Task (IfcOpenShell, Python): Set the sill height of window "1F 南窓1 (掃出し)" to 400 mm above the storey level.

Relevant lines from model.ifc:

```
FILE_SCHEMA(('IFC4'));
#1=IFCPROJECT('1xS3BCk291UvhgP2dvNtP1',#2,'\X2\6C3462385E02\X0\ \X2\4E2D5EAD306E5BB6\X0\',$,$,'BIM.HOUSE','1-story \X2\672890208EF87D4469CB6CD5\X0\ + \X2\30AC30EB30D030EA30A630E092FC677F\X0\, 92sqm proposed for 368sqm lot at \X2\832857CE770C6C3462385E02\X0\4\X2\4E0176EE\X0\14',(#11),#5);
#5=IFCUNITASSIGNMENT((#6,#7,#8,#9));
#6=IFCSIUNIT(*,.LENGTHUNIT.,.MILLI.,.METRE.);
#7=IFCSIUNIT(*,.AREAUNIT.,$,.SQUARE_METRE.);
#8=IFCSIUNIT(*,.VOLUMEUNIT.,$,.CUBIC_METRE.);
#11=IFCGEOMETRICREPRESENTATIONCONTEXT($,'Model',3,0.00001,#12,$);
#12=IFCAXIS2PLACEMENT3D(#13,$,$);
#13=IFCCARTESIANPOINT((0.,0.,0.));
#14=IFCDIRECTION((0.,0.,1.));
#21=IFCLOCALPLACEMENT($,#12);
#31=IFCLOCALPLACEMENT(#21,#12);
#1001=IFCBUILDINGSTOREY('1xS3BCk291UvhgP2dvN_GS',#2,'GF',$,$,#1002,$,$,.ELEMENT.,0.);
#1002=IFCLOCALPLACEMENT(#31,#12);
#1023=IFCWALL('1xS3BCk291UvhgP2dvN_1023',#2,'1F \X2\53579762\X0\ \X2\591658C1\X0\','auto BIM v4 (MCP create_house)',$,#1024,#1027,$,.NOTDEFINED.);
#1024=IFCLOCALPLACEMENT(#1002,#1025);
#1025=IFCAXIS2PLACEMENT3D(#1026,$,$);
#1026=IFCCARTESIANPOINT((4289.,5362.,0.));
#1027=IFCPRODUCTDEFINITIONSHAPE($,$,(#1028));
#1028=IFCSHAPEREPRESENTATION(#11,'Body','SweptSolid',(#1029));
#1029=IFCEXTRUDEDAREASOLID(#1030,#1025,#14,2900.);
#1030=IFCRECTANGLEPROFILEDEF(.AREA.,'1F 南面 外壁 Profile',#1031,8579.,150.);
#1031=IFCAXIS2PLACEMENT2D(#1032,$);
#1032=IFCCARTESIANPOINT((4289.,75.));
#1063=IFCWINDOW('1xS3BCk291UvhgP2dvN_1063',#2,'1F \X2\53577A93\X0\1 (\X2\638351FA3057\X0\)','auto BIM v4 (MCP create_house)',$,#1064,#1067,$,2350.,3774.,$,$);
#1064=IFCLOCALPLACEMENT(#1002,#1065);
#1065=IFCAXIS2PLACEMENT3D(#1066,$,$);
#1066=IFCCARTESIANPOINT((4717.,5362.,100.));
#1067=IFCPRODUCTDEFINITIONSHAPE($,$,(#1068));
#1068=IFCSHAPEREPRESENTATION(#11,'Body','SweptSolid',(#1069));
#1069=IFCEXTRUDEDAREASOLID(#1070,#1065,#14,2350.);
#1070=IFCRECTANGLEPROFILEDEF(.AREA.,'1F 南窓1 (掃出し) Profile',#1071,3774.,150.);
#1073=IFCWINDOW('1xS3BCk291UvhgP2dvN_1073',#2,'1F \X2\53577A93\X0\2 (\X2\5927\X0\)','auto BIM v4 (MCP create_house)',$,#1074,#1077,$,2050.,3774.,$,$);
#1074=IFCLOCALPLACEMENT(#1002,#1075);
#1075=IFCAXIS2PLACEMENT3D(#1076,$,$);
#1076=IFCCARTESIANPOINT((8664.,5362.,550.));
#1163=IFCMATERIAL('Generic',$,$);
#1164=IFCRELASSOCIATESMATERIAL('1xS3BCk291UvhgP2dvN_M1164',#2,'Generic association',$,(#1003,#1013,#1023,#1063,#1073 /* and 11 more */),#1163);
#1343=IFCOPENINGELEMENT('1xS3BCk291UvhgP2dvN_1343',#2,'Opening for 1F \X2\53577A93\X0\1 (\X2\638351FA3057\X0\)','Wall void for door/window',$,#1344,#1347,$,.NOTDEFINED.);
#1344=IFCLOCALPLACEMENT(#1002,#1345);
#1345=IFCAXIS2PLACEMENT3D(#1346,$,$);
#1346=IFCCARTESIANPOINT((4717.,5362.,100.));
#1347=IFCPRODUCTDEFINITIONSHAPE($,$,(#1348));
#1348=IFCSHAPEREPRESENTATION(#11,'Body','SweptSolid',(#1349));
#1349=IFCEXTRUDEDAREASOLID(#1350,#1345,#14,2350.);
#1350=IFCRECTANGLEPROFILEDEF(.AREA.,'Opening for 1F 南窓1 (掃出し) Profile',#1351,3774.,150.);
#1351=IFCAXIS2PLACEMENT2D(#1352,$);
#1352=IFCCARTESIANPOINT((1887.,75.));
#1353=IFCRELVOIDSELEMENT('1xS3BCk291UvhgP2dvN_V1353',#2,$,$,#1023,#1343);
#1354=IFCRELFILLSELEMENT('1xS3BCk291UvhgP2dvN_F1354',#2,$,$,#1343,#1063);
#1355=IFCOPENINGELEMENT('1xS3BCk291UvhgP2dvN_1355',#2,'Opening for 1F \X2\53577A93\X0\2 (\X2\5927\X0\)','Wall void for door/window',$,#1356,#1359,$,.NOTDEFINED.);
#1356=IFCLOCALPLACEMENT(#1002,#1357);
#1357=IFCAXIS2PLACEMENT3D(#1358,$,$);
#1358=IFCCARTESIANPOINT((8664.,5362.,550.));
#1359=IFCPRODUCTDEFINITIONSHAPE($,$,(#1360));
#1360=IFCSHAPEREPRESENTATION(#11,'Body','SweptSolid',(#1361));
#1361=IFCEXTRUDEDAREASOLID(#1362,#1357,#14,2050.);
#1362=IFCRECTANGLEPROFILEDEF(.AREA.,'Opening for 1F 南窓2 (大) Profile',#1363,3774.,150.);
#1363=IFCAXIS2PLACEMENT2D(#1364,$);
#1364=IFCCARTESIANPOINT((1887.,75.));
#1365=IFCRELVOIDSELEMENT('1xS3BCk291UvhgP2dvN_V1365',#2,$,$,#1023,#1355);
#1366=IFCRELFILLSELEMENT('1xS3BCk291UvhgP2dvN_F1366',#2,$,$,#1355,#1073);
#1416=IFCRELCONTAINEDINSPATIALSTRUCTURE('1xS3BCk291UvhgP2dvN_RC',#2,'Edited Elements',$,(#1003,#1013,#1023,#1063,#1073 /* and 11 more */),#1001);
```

```python
import numpy as np
import ifcopenshell
import ifcopenshell.api.geometry
import ifcopenshell.geom
import ifcopenshell.util.element
import ifcopenshell.util.placement
import ifcopenshell.util.shape
import ifcopenshell.util.unit

model = ifcopenshell.open("model.ifc")
unit_scale = ifcopenshell.util.unit.calculate_unit_scale(model)

window = model.by_guid("1xS3BCk291UvhgP2dvN_1063")
opening = window.FillsVoids[0].RelatingOpeningElement
storey = ifcopenshell.util.element.get_container(window, ifc_class="IfcBuildingStorey")
level = ifcopenshell.util.placement.get_local_placement(storey.ObjectPlacement)[2, 3]

# The opening's origin need not be at the sill, so measure its lowest point.
shape = ifcopenshell.geom.create_shape(ifcopenshell.geom.settings(), opening)
bottom = ifcopenshell.util.shape.get_shape_bottom_elevation(shape, shape.geometry) / unit_scale
dz = level + 400.0 - bottom

shift = np.array([0.0, 0.0, dz])
# The window is not placed relative to its opening, so move both.
for product in (opening, window):
    matrix = ifcopenshell.util.placement.get_local_placement(product.ObjectPlacement)
    matrix[:3, 3] += shift
    ifcopenshell.api.geometry.edit_object_placement(model, product=product, matrix=matrix, is_si=False)

print(f"moved by {dz * unit_scale:+.3f} m")

model.write("model_edited.ifc")
```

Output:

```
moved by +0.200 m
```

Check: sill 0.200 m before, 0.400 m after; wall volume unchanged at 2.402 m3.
